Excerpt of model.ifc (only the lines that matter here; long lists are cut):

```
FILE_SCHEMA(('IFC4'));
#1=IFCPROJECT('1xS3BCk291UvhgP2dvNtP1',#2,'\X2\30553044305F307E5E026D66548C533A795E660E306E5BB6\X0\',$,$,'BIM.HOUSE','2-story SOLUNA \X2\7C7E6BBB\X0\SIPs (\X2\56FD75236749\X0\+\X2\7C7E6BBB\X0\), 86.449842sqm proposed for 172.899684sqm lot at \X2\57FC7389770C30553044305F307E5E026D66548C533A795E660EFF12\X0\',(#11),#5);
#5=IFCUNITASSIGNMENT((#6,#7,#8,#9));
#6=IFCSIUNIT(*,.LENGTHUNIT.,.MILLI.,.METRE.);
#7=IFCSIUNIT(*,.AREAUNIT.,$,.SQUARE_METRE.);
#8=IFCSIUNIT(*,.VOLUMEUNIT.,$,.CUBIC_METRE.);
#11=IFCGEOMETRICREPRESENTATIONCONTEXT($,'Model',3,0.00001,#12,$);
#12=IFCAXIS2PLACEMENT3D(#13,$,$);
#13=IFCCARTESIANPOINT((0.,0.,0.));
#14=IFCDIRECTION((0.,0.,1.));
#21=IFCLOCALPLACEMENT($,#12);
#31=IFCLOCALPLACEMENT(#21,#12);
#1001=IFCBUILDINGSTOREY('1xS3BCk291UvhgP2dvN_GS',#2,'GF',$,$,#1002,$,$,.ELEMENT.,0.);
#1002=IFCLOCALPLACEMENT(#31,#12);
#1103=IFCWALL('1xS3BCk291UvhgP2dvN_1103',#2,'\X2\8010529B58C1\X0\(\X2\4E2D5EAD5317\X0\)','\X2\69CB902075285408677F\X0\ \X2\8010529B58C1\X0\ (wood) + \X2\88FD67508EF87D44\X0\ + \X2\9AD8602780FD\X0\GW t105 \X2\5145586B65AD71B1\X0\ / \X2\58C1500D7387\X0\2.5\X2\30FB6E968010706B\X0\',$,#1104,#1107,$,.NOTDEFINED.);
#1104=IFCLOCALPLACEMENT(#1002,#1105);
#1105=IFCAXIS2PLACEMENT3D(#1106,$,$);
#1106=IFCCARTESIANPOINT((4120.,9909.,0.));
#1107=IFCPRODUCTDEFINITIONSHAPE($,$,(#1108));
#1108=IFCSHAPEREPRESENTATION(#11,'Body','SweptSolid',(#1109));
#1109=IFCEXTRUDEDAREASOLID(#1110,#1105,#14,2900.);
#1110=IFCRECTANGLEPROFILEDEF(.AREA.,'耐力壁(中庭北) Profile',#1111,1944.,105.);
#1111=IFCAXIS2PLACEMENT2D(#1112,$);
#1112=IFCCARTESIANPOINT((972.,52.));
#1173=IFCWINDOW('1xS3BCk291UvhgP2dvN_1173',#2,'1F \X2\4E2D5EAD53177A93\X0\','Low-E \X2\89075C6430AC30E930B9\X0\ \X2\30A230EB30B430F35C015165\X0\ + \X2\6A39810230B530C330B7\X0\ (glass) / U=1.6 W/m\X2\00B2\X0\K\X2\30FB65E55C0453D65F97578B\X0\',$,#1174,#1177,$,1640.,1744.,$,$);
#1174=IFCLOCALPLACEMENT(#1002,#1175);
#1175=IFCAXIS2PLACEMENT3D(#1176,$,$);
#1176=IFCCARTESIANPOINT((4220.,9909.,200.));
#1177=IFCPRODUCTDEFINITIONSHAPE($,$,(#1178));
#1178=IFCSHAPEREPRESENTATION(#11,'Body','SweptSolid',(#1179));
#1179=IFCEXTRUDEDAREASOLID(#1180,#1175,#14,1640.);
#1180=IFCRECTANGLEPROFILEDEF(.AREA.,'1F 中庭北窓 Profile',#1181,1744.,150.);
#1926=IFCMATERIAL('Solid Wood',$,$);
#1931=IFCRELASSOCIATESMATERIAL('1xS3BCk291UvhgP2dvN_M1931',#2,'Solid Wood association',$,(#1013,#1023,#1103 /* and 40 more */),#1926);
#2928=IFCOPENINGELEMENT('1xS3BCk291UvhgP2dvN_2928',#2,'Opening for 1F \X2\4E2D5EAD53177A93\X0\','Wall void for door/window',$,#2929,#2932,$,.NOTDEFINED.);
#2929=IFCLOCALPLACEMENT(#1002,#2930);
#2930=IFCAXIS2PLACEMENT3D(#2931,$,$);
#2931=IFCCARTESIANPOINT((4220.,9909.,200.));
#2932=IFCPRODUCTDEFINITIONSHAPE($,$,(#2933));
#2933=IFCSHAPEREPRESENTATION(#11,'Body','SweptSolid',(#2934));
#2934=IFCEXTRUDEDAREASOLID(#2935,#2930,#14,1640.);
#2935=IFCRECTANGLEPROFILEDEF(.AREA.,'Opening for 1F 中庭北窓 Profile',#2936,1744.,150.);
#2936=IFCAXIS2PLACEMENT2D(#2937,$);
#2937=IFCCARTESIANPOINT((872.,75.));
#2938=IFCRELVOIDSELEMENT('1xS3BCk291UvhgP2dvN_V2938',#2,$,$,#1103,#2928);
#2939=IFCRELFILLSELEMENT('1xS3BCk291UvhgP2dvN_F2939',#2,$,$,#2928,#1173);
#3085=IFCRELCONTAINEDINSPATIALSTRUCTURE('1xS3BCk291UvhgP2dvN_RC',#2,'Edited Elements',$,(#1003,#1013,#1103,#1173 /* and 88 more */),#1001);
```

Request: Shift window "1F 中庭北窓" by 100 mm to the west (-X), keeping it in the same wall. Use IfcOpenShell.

```python
import ifcopenshell
import ifcopenshell.api.geometry
import ifcopenshell.util.placement

model = ifcopenshell.open("model.ifc")

window = model.by_guid("1xS3BCk291UvhgP2dvN_1173")
opening = window.FillsVoids[0].RelatingOpeningElement
wall = opening.VoidsElements[0].RelatingBuildingElement

wall_matrix = ifcopenshell.util.placement.get_local_placement(wall.ObjectPlacement)
shift = wall_matrix[:3, 0] * -100.0
before = ifcopenshell.util.placement.get_local_placement(window.ObjectPlacement)[:3, 3].copy()

# The window is not placed relative to its opening, so move both.
for product in (opening, window):
    matrix = ifcopenshell.util.placement.get_local_placement(product.ObjectPlacement)
    matrix[:3, 3] += shift
    ifcopenshell.api.geometry.edit_object_placement(model, product=product, matrix=matrix, is_si=False)

after = ifcopenshell.util.placement.get_local_placement(window.ObjectPlacement)[:3, 3]
print("window moved by", (after - before).round(3) + 0.0)

model.write("model_edited.ifc")
```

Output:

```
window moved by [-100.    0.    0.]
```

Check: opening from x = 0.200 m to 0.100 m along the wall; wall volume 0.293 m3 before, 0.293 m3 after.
